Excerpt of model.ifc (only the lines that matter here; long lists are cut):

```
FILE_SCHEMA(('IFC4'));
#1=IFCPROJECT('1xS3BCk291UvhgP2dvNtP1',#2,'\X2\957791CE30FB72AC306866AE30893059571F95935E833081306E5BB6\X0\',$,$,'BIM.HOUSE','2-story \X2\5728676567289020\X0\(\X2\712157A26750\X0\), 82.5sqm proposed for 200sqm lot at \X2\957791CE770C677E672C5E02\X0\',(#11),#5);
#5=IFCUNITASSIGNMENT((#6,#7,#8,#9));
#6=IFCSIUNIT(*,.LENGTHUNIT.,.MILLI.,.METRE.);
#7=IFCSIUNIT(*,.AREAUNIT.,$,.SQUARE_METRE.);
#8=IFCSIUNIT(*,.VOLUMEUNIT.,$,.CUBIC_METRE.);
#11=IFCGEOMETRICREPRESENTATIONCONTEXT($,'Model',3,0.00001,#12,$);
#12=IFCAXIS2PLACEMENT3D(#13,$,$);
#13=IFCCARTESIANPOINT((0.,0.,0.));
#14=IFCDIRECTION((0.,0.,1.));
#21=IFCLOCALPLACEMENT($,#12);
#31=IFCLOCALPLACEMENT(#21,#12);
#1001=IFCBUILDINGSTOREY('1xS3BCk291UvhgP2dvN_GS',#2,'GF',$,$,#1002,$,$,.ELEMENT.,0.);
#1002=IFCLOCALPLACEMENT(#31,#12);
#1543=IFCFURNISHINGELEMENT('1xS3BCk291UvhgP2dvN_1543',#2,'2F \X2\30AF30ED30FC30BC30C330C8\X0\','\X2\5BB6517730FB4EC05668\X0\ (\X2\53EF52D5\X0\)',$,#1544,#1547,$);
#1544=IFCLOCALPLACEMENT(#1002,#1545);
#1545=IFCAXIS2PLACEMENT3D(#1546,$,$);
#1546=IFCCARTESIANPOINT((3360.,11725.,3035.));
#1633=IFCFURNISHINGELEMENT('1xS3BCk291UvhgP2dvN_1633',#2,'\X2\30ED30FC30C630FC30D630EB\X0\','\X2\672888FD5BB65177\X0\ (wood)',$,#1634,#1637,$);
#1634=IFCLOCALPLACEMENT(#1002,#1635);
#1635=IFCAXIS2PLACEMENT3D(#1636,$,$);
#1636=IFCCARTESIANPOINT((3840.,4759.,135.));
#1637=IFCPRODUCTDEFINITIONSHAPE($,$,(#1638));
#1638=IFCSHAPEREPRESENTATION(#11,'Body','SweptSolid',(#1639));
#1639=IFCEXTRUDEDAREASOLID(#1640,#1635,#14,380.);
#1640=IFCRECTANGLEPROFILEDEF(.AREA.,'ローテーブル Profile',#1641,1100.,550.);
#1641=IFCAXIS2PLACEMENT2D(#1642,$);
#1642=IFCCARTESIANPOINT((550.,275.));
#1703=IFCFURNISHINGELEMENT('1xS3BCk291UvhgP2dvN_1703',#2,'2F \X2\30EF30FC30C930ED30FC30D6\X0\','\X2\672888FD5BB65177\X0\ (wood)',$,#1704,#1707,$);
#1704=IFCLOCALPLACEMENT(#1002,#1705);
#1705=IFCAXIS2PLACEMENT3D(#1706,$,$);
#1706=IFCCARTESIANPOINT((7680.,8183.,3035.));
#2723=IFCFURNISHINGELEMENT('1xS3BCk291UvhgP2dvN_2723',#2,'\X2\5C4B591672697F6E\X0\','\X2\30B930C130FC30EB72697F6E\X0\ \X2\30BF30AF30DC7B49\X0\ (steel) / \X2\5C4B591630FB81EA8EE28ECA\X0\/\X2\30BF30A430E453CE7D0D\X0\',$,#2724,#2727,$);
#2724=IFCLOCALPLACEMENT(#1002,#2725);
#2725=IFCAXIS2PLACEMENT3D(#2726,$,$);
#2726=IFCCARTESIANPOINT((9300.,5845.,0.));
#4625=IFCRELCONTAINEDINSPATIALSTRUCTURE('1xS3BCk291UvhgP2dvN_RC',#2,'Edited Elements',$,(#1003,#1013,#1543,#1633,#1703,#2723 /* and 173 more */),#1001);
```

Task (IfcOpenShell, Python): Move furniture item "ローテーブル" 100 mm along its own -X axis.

```python
import ifcopenshell
import ifcopenshell.api.geometry
import ifcopenshell.util.placement

model = ifcopenshell.open("model.ifc")

item = model.by_guid("1xS3BCk291UvhgP2dvN_1633")
matrix = ifcopenshell.util.placement.get_local_placement(item.ObjectPlacement)
matrix[:3, 3] -= matrix[:3, 0] * 100.0
ifcopenshell.api.geometry.edit_object_placement(model, product=item, matrix=matrix, is_si=False)

print(ifcopenshell.util.placement.get_local_placement(item.ObjectPlacement).round(3) + 0.0)

model.write("model_v2.ifc")
```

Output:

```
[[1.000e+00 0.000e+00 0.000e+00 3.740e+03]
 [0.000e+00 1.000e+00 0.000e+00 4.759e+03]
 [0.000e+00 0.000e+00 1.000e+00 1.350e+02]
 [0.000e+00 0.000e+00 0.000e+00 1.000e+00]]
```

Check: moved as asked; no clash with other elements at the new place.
